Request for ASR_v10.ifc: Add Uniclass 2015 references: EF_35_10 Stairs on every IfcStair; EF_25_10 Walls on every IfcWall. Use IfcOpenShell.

First a look at what the model holds.

```python
import ifcopenshell

model = ifcopenshell.open("ASR_v10.ifc")
print(model.schema)
print("classifications:", [c.Name for c in model.by_type("IfcClassification")])
for ifc_class in ("IfcDoor", "IfcRoof", "IfcStair", "IfcWall", "IfcWindow"):
    print(ifc_class, len(model.by_type(ifc_class)))
```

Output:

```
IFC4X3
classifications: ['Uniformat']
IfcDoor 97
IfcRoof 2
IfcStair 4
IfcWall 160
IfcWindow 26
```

```python
import ifcopenshell
import ifcopenshell.api.classification

model = ifcopenshell.open("ASR_v10.ifc")

system = ifcopenshell.api.classification.add_classification(model, classification="Uniclass 2015")

codes = {
    "IfcStair": ("EF_35_10", "Stairs"),
    "IfcWall": ("EF_25_10", "Walls"),
}
for ifc_class, (code, name) in codes.items():
    products = model.by_type(ifc_class)
    ifcopenshell.api.classification.add_reference(
        model, products=products, classification=system, identification=code, name=name
    )
    print(code, len(products))

model.write("ASR_v10_v2.ifc")
```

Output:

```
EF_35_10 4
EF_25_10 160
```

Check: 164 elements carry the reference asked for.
